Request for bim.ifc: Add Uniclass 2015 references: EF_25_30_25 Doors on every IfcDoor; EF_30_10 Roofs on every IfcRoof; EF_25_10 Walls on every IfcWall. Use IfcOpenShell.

First a look at what the model holds.

```python
import ifcopenshell

model = ifcopenshell.open("bim.ifc")
print(model.schema)
print("classifications:", [c.Name for c in model.by_type("IfcClassification")])
for ifc_class in ("IfcDoor", "IfcRoof", "IfcStair", "IfcWall", "IfcWindow"):
    print(ifc_class, len(model.by_type(ifc_class)))
```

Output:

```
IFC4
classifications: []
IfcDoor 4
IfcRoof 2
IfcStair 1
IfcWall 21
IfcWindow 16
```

```python
import ifcopenshell
import ifcopenshell.api.classification

model = ifcopenshell.open("bim.ifc")

system = ifcopenshell.api.classification.add_classification(model, classification="Uniclass 2015")

codes = {
    "IfcDoor": ("EF_25_30_25", "Doors"),
    "IfcRoof": ("EF_30_10", "Roofs"),
    "IfcWall": ("EF_25_10", "Walls"),
}
for ifc_class, (code, name) in codes.items():
    products = model.by_type(ifc_class)
    ifcopenshell.api.classification.add_reference(
        model, products=products, classification=system, identification=code, name=name
    )
    print(code, len(products))

model.write("bim_edited.ifc")
```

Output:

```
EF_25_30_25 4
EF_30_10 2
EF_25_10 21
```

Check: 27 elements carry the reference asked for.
